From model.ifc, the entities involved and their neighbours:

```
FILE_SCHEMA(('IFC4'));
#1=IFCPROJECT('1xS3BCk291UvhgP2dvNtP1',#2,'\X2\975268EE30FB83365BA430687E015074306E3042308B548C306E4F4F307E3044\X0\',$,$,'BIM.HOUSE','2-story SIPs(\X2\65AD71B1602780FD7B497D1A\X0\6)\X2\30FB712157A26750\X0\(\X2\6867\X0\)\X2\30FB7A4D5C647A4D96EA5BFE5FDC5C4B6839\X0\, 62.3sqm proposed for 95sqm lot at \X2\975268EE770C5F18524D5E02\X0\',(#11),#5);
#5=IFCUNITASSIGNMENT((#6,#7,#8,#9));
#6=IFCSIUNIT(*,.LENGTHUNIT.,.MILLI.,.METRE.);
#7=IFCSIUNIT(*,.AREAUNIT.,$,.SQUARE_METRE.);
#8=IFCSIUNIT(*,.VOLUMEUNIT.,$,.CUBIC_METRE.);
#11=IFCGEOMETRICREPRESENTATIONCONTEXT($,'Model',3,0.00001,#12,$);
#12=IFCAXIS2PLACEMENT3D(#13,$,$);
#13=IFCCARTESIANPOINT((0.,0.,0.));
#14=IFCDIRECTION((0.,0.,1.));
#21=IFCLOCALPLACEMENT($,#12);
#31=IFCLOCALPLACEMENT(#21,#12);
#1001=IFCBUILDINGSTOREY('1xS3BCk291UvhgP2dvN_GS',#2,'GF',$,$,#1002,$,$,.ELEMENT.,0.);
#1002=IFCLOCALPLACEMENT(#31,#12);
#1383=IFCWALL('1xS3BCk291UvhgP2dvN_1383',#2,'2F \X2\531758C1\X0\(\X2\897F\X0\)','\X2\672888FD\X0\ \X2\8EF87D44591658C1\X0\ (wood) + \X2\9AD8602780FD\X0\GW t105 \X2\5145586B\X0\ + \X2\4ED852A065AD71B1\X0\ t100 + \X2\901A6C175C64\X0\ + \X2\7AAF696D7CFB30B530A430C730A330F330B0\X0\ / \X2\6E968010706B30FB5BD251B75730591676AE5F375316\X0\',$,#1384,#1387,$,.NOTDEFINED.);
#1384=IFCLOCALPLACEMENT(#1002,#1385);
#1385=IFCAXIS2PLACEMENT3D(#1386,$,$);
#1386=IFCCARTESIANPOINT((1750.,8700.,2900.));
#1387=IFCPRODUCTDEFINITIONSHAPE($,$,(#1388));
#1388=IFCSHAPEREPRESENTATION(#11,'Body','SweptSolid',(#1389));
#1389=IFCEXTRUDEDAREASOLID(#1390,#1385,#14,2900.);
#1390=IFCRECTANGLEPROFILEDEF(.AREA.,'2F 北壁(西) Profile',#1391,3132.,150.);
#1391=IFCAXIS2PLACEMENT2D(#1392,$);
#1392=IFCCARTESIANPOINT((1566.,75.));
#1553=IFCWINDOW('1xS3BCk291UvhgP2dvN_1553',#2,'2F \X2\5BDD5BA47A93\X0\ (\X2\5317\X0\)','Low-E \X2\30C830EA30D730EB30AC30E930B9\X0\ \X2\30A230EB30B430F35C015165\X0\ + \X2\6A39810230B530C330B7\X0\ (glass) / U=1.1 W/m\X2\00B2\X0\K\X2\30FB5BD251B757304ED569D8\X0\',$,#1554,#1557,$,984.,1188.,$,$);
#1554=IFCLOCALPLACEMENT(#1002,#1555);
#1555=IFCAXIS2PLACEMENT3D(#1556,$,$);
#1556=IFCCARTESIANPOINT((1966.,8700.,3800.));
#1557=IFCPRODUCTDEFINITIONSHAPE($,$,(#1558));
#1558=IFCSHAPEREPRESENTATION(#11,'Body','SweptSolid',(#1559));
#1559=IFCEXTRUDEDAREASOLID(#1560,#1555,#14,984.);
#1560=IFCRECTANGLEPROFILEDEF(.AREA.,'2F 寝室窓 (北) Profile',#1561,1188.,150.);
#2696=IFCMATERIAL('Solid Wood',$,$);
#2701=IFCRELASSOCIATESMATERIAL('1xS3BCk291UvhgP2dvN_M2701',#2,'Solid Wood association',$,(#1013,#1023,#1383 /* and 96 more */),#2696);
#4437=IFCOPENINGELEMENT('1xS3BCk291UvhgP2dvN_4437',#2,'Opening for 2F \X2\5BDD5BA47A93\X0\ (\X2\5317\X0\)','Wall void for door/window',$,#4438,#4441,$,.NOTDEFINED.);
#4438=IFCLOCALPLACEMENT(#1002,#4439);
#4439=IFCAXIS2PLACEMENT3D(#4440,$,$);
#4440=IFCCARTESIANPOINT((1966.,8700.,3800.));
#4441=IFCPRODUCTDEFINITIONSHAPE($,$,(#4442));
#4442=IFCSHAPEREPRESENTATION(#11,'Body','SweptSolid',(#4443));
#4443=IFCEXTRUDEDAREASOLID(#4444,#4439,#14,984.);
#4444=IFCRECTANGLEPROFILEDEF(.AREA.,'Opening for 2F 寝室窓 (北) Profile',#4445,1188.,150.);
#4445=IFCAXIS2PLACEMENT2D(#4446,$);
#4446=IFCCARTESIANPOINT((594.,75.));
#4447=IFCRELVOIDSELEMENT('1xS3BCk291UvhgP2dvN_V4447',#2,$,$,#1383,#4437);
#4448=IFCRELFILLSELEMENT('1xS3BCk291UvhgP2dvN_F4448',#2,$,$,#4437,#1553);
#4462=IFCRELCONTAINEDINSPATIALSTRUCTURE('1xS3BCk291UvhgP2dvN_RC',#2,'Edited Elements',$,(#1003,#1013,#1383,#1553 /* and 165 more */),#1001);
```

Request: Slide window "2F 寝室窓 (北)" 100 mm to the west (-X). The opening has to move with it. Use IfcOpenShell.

```python
import ifcopenshell
import ifcopenshell.api.geometry
import ifcopenshell.util.placement

model = ifcopenshell.open("model.ifc")

window = model.by_guid("1xS3BCk291UvhgP2dvN_1553")
opening = window.FillsVoids[0].RelatingOpeningElement
wall = opening.VoidsElements[0].RelatingBuildingElement

wall_matrix = ifcopenshell.util.placement.get_local_placement(wall.ObjectPlacement)
shift = wall_matrix[:3, 0] * -100.0
before = ifcopenshell.util.placement.get_local_placement(window.ObjectPlacement)[:3, 3].copy()

# The window is not placed relative to its opening, so move both.
for product in (opening, window):
    matrix = ifcopenshell.util.placement.get_local_placement(product.ObjectPlacement)
    matrix[:3, 3] += shift
    ifcopenshell.api.geometry.edit_object_placement(model, product=product, matrix=matrix, is_si=False)

after = ifcopenshell.util.placement.get_local_placement(window.ObjectPlacement)[:3, 3]
print("window moved by", (after - before).round(3) + 0.0)

model.write("model_updated.ifc")
```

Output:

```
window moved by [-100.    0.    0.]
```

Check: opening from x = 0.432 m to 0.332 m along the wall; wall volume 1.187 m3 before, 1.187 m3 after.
